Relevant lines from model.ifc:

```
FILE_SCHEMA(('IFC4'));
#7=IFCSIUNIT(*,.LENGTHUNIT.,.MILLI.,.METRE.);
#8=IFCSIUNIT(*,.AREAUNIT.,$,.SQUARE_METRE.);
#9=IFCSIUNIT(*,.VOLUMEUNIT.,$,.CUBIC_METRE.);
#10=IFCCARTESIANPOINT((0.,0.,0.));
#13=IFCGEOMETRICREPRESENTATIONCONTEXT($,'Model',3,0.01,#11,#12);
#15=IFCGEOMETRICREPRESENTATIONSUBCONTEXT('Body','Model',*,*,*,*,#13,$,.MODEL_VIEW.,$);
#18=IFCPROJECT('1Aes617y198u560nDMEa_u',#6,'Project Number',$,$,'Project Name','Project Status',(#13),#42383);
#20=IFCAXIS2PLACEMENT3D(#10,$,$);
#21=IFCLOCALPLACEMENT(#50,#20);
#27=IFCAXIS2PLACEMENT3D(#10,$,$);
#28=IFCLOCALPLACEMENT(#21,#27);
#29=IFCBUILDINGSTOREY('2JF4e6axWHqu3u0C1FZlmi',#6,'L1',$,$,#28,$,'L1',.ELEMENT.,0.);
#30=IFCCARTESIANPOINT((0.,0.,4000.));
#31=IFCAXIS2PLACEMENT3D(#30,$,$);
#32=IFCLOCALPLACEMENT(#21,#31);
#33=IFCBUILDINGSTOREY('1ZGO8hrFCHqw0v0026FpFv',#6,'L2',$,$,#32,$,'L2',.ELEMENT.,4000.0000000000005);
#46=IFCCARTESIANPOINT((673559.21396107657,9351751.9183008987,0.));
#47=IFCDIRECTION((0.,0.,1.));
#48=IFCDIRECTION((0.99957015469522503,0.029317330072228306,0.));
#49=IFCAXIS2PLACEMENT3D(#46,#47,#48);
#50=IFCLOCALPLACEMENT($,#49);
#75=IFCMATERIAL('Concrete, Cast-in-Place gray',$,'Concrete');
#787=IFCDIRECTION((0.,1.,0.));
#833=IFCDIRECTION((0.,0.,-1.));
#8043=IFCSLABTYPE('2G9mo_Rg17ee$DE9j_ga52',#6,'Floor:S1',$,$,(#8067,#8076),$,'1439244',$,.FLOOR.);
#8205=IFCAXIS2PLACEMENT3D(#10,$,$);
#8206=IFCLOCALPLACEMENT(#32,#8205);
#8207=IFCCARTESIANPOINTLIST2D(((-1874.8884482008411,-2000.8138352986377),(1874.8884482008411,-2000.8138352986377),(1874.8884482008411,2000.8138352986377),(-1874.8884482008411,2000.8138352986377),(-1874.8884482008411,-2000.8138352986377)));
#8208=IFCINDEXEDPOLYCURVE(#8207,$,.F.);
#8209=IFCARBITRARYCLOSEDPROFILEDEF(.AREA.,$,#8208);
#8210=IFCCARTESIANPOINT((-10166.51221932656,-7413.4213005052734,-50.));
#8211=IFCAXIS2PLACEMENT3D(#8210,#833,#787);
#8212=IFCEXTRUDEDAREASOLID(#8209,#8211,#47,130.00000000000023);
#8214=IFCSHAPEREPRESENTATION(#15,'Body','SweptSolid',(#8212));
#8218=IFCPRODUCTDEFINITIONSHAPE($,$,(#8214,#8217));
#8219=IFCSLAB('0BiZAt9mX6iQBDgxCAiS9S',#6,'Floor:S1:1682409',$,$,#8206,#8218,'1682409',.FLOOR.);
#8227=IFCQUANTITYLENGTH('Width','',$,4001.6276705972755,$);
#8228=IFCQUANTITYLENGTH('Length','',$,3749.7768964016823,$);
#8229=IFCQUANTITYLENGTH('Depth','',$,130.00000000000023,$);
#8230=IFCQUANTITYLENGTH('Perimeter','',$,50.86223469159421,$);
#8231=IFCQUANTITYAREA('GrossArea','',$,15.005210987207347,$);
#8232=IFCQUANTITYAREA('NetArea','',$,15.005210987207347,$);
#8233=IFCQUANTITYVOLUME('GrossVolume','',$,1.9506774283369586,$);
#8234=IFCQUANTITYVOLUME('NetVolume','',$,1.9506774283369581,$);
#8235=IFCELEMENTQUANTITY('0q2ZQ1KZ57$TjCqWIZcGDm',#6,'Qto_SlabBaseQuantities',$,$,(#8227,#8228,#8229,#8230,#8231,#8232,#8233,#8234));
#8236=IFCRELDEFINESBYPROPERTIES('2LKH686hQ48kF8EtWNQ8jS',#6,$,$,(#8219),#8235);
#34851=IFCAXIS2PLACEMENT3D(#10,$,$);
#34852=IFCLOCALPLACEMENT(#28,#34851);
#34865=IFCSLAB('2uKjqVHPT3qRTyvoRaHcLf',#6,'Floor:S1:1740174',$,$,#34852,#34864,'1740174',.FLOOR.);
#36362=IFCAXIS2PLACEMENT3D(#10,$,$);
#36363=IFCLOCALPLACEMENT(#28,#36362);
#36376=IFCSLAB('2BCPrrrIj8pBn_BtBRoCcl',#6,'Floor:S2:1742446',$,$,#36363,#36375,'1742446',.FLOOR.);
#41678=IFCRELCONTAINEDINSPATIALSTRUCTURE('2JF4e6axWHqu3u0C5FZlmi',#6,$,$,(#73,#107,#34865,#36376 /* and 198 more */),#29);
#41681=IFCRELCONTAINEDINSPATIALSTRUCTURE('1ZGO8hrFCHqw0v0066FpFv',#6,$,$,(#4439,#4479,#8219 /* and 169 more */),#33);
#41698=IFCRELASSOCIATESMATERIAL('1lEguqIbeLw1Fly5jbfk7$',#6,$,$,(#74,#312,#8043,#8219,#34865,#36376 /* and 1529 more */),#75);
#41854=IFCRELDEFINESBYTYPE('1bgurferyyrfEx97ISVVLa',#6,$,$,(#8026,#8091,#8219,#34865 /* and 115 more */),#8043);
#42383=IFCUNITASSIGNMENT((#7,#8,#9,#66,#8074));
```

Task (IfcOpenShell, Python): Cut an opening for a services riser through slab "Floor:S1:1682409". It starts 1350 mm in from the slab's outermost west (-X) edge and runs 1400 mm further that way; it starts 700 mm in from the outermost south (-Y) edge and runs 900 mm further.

```python
import numpy as np
import ifcopenshell
import ifcopenshell.api.feature
import ifcopenshell.api.geometry
import ifcopenshell.api.pset
import ifcopenshell.api.root
import ifcopenshell.geom
import ifcopenshell.util.element
import ifcopenshell.util.placement
import ifcopenshell.util.representation
import ifcopenshell.util.shape
import ifcopenshell.util.unit

model = ifcopenshell.open("model.ifc")
unit_scale = ifcopenshell.util.unit.calculate_unit_scale(model)
area_scale = ifcopenshell.util.unit.calculate_unit_scale(model, "AREAUNIT")
volume_scale = ifcopenshell.util.unit.calculate_unit_scale(model, "VOLUMEUNIT")
settings = ifcopenshell.geom.settings()


def volume(element):
    """Net volume in cubic metres, openings subtracted."""
    shape = ifcopenshell.geom.create_shape(settings, element)
    return ifcopenshell.util.shape.get_volume(shape.geometry)


slab = model.by_guid("0BiZAt9mX6iQBDgxCAiS9S")
before = volume(slab)

# Extent in the slab's own axes, in metres. The edges named are its -X and -Y sides.
slab_shape = ifcopenshell.geom.create_shape(settings, slab)
vertices = ifcopenshell.util.shape.get_vertices(slab_shape.geometry)
x_min, y_min, bottom = vertices.min(axis=0)
top = vertices[:, 2].max()

opening = ifcopenshell.api.root.create_entity(model, ifc_class="IfcOpeningElement", name="Services riser opening", predefined_type="OPENING")
context = ifcopenshell.util.representation.get_context(model, "Model", "Body", "MODEL_VIEW")
width, depth = 1.4, 0.9
outline = [(0.0, 0.0), (width, 0.0), (width, depth), (0.0, depth), (0.0, 0.0)]
# Overshoot both faces by 50 mm so the cut is clean.
shape = ifcopenshell.api.geometry.add_slab_representation(
    model, context=context, depth=top - bottom + 0.1, polyline=outline
)
ifcopenshell.api.geometry.assign_representation(model, product=opening, representation=shape)

matrix = ifcopenshell.util.placement.get_local_placement(slab.ObjectPlacement)
matrix[:, 3] = matrix @ np.append(np.array([x_min + 1.35, y_min + 0.7, bottom - 0.05]) / unit_scale, 1.0)
ifcopenshell.api.geometry.edit_object_placement(model, product=opening, matrix=matrix, is_si=False)
ifcopenshell.api.feature.add_feature(model, feature=opening, element=slab)

after = volume(slab)

# Update the slab's stored quantities.
qto = model.by_id(ifcopenshell.util.element.get_pset(slab, "Qto_SlabBaseQuantities", should_inherit=False)["id"])
ifcopenshell.api.pset.edit_qto(model, qto=qto, properties={
    "NetArea": after / (top - bottom) / area_scale,
    "NetVolume": after / volume_scale,
})

print(f"slab volume {before:.3f} -> {after:.3f} m3")

model.write("model_updated.ifc")
```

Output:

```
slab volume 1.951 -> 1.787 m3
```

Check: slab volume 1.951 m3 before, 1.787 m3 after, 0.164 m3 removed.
